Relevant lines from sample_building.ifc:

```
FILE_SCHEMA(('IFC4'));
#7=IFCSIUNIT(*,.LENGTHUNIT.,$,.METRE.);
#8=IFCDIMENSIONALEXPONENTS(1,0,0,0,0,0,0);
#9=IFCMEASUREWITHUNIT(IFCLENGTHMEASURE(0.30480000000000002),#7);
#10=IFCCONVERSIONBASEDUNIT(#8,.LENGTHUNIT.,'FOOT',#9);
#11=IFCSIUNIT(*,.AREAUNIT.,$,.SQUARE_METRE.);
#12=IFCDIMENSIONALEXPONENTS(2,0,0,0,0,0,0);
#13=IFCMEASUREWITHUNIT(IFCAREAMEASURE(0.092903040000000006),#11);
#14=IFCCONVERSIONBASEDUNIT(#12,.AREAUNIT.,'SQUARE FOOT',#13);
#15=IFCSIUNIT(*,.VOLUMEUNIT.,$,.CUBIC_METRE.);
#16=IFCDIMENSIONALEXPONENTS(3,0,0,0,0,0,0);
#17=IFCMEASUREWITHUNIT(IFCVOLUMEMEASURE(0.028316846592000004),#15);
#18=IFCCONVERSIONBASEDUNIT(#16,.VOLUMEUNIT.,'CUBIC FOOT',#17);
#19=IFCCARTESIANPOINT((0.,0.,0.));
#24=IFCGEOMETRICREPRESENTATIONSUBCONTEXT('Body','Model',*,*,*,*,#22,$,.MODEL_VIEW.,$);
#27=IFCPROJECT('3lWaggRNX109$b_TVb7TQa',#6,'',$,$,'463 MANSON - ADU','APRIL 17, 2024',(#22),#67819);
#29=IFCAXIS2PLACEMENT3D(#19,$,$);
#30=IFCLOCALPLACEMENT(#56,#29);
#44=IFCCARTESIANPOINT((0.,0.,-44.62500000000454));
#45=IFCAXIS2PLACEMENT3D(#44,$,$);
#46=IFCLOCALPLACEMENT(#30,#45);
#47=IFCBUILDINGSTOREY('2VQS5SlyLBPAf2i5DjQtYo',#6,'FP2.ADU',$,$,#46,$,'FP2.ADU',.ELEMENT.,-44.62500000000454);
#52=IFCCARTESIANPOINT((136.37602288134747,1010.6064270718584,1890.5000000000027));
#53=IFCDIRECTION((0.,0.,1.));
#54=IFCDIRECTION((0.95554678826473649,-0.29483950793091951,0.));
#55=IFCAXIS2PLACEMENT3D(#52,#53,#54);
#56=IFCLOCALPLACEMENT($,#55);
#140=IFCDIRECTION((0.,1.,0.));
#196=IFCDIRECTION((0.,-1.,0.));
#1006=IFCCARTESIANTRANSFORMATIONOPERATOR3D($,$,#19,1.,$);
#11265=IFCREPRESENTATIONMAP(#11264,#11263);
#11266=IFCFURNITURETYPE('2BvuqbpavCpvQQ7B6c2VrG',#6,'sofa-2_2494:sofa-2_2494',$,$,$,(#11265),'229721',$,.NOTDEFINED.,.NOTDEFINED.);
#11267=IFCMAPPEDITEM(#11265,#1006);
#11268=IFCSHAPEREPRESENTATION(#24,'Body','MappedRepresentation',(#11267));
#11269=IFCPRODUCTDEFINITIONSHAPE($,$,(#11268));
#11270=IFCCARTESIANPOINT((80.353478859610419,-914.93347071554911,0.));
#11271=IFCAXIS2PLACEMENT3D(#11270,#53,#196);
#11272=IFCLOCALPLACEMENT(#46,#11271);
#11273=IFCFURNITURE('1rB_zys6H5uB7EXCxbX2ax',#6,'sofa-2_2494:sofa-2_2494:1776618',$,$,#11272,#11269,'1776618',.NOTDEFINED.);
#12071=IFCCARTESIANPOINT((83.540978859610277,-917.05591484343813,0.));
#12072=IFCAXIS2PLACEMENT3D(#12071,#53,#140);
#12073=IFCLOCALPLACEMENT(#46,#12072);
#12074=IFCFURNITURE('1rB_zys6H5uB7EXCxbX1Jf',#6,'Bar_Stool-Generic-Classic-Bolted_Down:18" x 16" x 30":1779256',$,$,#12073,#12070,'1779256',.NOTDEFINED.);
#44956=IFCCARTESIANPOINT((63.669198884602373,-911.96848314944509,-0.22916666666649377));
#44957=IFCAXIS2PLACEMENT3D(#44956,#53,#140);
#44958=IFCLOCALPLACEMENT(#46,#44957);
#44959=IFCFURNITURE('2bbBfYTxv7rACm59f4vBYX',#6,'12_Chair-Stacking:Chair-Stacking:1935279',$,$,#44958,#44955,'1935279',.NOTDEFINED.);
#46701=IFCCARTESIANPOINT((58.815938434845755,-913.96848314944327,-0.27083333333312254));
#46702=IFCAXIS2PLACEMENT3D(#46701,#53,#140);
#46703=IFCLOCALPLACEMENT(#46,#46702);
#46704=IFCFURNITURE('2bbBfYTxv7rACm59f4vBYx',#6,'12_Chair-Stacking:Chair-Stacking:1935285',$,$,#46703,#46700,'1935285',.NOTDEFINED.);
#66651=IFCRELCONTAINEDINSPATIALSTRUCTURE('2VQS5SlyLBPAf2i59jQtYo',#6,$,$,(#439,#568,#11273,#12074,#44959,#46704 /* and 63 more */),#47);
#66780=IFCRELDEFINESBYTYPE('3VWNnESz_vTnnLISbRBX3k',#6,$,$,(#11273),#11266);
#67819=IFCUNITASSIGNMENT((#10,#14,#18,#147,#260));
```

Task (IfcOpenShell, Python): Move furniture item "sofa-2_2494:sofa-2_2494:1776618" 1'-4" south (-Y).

```python
import ifcopenshell
import ifcopenshell.api.geometry
import ifcopenshell.util.placement
import ifcopenshell.util.unit

model = ifcopenshell.open("sample_building.ifc")
unit_scale = ifcopenshell.util.unit.calculate_unit_scale(model)

item = model.by_guid("1rB_zys6H5uB7EXCxbX2ax")
matrix = ifcopenshell.util.placement.get_local_placement(item.ObjectPlacement)
matrix[1, 3] -= 16 * 0.0254 / unit_scale
ifcopenshell.api.geometry.edit_object_placement(model, product=item, matrix=matrix, is_si=False)

print(ifcopenshell.util.placement.get_local_placement(item.ObjectPlacement).round(3) + 0.0)

model.write("sample_building_rev.ifc")
```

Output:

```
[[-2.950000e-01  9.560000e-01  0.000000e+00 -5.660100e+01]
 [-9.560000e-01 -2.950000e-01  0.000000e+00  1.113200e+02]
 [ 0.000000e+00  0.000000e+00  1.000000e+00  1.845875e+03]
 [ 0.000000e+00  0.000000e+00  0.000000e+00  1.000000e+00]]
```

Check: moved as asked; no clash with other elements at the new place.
